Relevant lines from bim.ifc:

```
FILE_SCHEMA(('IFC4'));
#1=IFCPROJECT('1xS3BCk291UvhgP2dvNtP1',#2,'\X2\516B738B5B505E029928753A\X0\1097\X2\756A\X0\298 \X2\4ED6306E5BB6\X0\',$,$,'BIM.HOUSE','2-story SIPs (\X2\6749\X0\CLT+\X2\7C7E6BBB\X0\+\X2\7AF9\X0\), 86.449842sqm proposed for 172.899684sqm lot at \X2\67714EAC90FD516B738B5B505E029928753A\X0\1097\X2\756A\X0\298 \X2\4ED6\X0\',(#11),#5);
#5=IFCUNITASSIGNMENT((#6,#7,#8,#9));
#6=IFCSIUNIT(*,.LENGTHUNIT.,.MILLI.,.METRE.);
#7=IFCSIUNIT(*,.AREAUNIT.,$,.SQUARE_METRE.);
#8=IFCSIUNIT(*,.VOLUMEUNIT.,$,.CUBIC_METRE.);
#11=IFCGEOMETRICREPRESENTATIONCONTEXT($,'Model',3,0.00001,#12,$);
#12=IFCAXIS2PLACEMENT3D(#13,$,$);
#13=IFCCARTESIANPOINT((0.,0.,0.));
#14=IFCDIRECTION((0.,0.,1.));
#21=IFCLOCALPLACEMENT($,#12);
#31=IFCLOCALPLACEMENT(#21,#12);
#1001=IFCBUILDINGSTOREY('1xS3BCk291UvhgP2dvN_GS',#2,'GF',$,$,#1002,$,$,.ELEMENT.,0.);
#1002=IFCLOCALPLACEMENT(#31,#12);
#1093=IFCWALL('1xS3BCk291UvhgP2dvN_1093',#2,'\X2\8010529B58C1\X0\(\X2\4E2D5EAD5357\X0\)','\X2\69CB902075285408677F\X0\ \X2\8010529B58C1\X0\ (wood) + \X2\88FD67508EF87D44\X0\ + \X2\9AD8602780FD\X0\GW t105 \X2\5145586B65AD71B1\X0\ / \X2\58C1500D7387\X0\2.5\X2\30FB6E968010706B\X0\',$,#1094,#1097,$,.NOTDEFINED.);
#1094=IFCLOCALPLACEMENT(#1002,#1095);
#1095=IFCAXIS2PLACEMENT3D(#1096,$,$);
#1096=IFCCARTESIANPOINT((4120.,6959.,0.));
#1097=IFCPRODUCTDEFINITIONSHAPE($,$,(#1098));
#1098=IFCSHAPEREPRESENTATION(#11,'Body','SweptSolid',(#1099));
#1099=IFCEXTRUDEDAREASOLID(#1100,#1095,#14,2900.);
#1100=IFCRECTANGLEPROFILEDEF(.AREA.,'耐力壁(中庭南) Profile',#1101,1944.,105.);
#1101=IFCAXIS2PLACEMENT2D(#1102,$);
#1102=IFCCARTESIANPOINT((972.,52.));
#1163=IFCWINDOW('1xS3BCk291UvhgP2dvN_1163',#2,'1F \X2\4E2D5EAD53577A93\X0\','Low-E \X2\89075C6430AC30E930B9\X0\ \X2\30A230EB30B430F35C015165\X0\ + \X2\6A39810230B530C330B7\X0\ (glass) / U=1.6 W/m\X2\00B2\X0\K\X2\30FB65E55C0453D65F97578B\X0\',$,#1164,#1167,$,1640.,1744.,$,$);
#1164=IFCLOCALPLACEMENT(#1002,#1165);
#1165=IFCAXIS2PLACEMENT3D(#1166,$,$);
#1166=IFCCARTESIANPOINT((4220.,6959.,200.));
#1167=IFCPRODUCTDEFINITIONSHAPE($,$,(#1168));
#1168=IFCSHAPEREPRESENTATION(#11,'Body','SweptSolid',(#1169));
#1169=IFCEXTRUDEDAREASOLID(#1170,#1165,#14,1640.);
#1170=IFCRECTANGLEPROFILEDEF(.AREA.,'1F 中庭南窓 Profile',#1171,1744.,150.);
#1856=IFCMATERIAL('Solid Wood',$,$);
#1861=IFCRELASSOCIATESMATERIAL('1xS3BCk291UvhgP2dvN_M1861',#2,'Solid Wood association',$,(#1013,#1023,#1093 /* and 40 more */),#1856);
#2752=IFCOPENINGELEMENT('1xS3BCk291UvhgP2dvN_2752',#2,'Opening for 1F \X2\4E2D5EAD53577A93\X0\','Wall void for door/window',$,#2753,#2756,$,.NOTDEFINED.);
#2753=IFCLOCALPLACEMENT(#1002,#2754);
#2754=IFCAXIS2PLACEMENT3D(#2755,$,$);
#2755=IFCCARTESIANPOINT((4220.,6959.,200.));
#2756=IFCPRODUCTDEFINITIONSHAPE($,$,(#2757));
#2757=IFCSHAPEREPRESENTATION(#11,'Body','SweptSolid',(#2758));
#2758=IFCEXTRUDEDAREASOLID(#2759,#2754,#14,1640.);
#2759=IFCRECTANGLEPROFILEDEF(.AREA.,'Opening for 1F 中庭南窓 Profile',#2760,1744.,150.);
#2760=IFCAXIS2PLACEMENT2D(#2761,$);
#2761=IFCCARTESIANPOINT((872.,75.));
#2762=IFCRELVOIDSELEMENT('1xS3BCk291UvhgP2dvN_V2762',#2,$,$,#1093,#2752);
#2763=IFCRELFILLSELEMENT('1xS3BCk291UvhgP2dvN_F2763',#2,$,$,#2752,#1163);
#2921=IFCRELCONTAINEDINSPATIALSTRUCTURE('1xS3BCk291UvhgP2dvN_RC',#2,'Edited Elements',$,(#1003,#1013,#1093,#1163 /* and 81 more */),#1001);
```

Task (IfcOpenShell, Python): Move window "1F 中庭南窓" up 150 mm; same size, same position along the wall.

```python
import numpy as np
import ifcopenshell
import ifcopenshell.api.geometry
import ifcopenshell.util.placement
import ifcopenshell.util.unit

model = ifcopenshell.open("bim.ifc")
unit_scale = ifcopenshell.util.unit.calculate_unit_scale(model)

window = model.by_guid("1xS3BCk291UvhgP2dvN_1163")
opening = window.FillsVoids[0].RelatingOpeningElement
dz = 0.15 / unit_scale

shift = np.array([0.0, 0.0, dz])
# The window is not placed relative to its opening, so move both.
for product in (opening, window):
    matrix = ifcopenshell.util.placement.get_local_placement(product.ObjectPlacement)
    matrix[:3, 3] += shift
    ifcopenshell.api.geometry.edit_object_placement(model, product=product, matrix=matrix, is_si=False)

print(f"moved by {dz * unit_scale:+.3f} m")

model.write("bim_updated.ifc")
```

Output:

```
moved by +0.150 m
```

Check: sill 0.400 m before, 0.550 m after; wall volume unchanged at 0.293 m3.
